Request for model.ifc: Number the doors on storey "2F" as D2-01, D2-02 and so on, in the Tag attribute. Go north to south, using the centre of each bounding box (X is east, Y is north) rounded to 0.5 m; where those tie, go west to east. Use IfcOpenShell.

First a look at what the model holds.

```python
import ifcopenshell
import ifcopenshell.util.element
import ifcopenshell.util.placement

model = ifcopenshell.open("model.ifc")
print(model.schema)
storey = next(s for s in model.by_type("IfcBuildingStorey") if s.Name == "2F")
doors = [e for e in ifcopenshell.util.element.get_decomposition(storey) if e.is_a("IfcDoor")]
for e in sorted(doors, key=lambda e: e.id()):
    origin = ifcopenshell.util.placement.get_local_placement(e.ObjectPlacement)[:3, 3]
    print(e.id(), e.Tag, e.Name, origin.round(2) + 0.0, sep=" | ")
```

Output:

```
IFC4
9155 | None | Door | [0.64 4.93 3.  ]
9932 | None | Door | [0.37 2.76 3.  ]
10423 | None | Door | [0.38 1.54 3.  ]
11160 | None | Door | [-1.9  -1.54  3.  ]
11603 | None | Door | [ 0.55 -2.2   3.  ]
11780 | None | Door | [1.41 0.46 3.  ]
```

```python
import ifcopenshell
import ifcopenshell.geom
import ifcopenshell.util.element
import ifcopenshell.util.shape

model = ifcopenshell.open("model.ifc")
settings = ifcopenshell.geom.settings()
settings.set("use-world-coords", True)


def centre(element):
    shape = ifcopenshell.geom.create_shape(settings, element)
    return ifcopenshell.util.shape.get_bbox_centroid(shape.geometry)


storey = next(s for s in model.by_type("IfcBuildingStorey") if s.Name == "2F")
doors = [e for e in ifcopenshell.util.element.get_decomposition(storey) if e.is_a("IfcDoor")]

# Insertion points can sit at a corner or the storey origin, so sort by the geometry (in metres).
centres = {e: centre(e) for e in doors}
doors.sort(key=lambda e: (-round(centres[e][1] / 0.5), centres[e][0]))

for i, e in enumerate(doors, start=1):
    number = f"D2-{i:02d}"
    e.Tag = number
    print(e.id(), number)

model.write("model-out.ifc")
```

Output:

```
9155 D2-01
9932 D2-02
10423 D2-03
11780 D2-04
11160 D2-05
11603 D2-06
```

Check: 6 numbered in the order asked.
